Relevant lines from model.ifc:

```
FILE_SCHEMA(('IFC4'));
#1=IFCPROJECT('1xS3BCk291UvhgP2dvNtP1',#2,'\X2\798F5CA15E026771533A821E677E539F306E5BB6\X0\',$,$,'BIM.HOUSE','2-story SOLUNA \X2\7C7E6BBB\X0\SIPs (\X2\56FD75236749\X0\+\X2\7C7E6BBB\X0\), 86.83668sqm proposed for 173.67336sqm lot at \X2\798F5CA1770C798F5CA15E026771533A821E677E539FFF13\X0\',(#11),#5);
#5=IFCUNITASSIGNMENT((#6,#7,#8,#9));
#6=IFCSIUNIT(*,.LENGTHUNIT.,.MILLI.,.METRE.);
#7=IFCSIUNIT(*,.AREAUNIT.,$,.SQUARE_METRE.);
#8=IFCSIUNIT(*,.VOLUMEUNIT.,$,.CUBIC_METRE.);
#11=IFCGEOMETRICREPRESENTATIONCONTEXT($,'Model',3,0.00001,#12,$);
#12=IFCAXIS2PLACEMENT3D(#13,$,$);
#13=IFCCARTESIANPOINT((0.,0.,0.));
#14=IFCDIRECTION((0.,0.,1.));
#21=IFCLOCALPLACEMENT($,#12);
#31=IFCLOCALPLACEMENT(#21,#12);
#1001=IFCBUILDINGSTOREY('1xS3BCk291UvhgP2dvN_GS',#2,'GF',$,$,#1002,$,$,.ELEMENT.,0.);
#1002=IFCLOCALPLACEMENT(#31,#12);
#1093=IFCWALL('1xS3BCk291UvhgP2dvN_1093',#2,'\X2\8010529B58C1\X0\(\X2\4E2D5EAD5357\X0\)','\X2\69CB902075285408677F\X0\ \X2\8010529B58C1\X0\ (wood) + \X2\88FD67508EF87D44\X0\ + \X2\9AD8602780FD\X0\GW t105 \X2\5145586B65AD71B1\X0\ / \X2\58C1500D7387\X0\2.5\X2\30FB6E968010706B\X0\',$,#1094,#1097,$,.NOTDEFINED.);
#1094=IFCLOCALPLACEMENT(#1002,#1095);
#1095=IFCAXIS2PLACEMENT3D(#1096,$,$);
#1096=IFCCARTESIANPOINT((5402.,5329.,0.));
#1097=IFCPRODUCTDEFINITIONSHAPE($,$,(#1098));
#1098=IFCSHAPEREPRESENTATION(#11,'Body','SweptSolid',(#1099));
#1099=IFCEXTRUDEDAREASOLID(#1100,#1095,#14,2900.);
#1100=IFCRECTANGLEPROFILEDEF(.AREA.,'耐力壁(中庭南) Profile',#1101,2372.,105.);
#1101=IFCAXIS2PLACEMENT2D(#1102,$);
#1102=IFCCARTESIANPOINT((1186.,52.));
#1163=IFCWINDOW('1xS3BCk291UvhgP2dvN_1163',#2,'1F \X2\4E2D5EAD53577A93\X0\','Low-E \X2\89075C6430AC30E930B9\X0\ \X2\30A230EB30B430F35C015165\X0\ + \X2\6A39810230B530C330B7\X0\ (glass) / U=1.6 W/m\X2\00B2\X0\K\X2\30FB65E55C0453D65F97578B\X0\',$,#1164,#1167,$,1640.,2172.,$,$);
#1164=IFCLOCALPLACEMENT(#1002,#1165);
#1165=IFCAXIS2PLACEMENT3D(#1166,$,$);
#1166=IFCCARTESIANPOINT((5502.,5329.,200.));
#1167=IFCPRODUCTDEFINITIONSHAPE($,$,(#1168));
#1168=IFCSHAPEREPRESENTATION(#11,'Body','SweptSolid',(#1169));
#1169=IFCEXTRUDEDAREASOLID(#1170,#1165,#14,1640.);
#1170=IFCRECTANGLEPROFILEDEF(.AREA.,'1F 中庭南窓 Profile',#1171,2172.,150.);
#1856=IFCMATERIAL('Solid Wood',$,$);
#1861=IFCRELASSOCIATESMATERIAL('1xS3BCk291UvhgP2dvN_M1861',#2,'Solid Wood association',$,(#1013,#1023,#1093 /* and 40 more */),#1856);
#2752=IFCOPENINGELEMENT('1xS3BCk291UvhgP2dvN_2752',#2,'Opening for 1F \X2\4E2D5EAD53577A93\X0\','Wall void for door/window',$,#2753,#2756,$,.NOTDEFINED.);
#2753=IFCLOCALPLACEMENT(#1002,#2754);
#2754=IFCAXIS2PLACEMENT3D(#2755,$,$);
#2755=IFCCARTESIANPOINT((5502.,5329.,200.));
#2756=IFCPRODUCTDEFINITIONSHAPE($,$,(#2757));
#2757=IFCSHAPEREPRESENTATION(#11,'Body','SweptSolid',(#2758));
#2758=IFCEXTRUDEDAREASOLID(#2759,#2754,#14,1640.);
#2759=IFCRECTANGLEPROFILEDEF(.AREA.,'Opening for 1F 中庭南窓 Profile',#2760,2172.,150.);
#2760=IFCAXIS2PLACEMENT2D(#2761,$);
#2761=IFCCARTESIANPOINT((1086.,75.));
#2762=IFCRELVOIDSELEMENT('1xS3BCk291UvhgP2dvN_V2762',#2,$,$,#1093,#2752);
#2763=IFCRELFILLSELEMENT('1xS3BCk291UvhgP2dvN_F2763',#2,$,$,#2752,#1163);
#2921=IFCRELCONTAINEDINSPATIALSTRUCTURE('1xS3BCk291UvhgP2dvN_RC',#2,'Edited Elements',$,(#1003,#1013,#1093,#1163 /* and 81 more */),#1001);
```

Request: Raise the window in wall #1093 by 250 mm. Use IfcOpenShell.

```python
import numpy as np
import ifcopenshell
import ifcopenshell.api.geometry
import ifcopenshell.util.placement
import ifcopenshell.util.unit

model = ifcopenshell.open("model.ifc")
unit_scale = ifcopenshell.util.unit.calculate_unit_scale(model)

window = model.by_guid("1xS3BCk291UvhgP2dvN_1163")
opening = window.FillsVoids[0].RelatingOpeningElement
dz = 250.0

shift = np.array([0.0, 0.0, dz])
# The window is not placed relative to its opening, so move both.
for product in (opening, window):
    matrix = ifcopenshell.util.placement.get_local_placement(product.ObjectPlacement)
    matrix[:3, 3] += shift
    ifcopenshell.api.geometry.edit_object_placement(model, product=product, matrix=matrix, is_si=False)

print(f"moved by {dz * unit_scale:+.3f} m")

model.write("model_v2.ifc")
```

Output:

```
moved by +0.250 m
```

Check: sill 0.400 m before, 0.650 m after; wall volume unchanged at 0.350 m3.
